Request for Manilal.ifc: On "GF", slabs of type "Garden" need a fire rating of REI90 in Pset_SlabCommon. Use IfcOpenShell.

First a look at what the model holds.

```python
import ifcopenshell
import ifcopenshell.util.element

model = ifcopenshell.open("Manilal.ifc")
print(model.schema)
storey = next(s for s in model.by_type("IfcBuildingStorey") if s.Name == "GF")
slabs = [e for e in ifcopenshell.util.element.get_decomposition(storey) if e.is_a("IfcSlab")]
seen = {}
for e in slabs:
    element_type = ifcopenshell.util.element.get_type(e)
    key = (element_type.Name if element_type != e and element_type else None, ifcopenshell.util.element.get_pset(e, "Pset_SlabCommon", "FireRating"))
    seen[key] = seen.get(key, 0) + 1
for (name, value), count in sorted(seen.items(), key=str):
    print(count, "x", name, "|", value)
```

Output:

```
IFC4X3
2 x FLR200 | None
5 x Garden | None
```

```python
import ifcopenshell
import ifcopenshell.api.pset
import ifcopenshell.util.element

model = ifcopenshell.open("Manilal.ifc")

storey = next(s for s in model.by_type("IfcBuildingStorey") if s.Name == "GF")
slabs = [e for e in ifcopenshell.util.element.get_decomposition(storey) if e.is_a("IfcSlab")]

count = 0
for e in slabs:
    element_type = ifcopenshell.util.element.get_type(e)
    if element_type in (None, e) or element_type.Name != "Garden":
        continue
    # add_pset returns the element's existing set when there is one.
    pset = ifcopenshell.api.pset.add_pset(model, product=e, name="Pset_SlabCommon")
    ifcopenshell.api.pset.edit_pset(model, pset=pset, properties={"FireRating": "REI90"})
    count += 1

print(count, "slabs updated")

model.write("Manilal_rev.ifc")
```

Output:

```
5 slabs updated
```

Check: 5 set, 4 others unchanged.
